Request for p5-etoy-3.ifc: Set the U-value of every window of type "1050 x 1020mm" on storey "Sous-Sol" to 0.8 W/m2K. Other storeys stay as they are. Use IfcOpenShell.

First a look at what the model holds.

```python
import ifcopenshell
import ifcopenshell.util.element

model = ifcopenshell.open("p5-etoy-3.ifc")
print(model.schema)
storey = next(s for s in model.by_type("IfcBuildingStorey") if s.Name == "Sous-Sol")
windows = [e for e in ifcopenshell.util.element.get_decomposition(storey) if e.is_a("IfcWindow")]
seen = {}
for e in windows:
    element_type = ifcopenshell.util.element.get_type(e)
    key = (element_type.Name if element_type != e and element_type else None, ifcopenshell.util.element.get_pset(e, "Pset_WindowCommon", "ThermalTransmittance"))
    seen[key] = seen.get(key, 0) + 1
for (name, value), count in sorted(seen.items(), key=str):
    print(count, "x", name, "|", value)
```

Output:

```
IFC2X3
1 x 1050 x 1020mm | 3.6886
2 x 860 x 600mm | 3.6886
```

```python
import ifcopenshell
import ifcopenshell.api.pset
import ifcopenshell.util.element

model = ifcopenshell.open("p5-etoy-3.ifc")

storey = next(s for s in model.by_type("IfcBuildingStorey") if s.Name == "Sous-Sol")
windows = [e for e in ifcopenshell.util.element.get_decomposition(storey) if e.is_a("IfcWindow")]

count = 0
for e in windows:
    element_type = ifcopenshell.util.element.get_type(e)
    if element_type in (None, e) or element_type.Name != "1050 x 1020mm":
        continue
    # add_pset returns the element's existing set when there is one.
    pset = ifcopenshell.api.pset.add_pset(model, product=e, name="Pset_WindowCommon")
    ifcopenshell.api.pset.edit_pset(model, pset=pset, properties={"ThermalTransmittance": 0.8})
    count += 1

print(count, "windows updated")

model.write("p5-etoy-3_v2.ifc")
```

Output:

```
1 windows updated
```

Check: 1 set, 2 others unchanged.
